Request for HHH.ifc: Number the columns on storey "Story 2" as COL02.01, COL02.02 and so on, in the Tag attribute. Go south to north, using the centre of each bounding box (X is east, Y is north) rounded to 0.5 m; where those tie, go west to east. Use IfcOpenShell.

First a look at what the model holds.

```python
import ifcopenshell
import ifcopenshell.util.element
import ifcopenshell.util.placement

model = ifcopenshell.open("HHH.ifc")
print(model.schema)
storey = next(s for s in model.by_type("IfcBuildingStorey") if s.Name == "Story 2")
columns = [e for e in ifcopenshell.util.element.get_decomposition(storey) if e.is_a("IfcColumn")]
for e in sorted(columns, key=lambda e: e.id()):
    origin = ifcopenshell.util.placement.get_local_placement(e.ObjectPlacement)[:3, 3]
    print(e.id(), e.Tag, e.Name, origin.round(2) + 0.0, sep=" | ")
```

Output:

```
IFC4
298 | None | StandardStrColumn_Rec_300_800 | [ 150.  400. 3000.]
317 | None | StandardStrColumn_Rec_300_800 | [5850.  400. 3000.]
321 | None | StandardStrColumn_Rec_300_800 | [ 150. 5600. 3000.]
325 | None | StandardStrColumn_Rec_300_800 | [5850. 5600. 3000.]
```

```python
import ifcopenshell
import ifcopenshell.geom
import ifcopenshell.util.element
import ifcopenshell.util.shape

model = ifcopenshell.open("HHH.ifc")
settings = ifcopenshell.geom.settings()
settings.set("use-world-coords", True)


def centre(element):
    shape = ifcopenshell.geom.create_shape(settings, element)
    return ifcopenshell.util.shape.get_bbox_centroid(shape.geometry)


storey = next(s for s in model.by_type("IfcBuildingStorey") if s.Name == "Story 2")
columns = [e for e in ifcopenshell.util.element.get_decomposition(storey) if e.is_a("IfcColumn")]

# Insertion points can sit at a corner or the storey origin, so sort by the geometry (in metres).
centres = {e: centre(e) for e in columns}
columns.sort(key=lambda e: (round(centres[e][1] / 0.5), centres[e][0]))

for i, e in enumerate(columns, start=1):
    number = f"COL02.{i:02d}"
    e.Tag = number
    print(e.id(), number)

model.write("HHH_v2.ifc")
```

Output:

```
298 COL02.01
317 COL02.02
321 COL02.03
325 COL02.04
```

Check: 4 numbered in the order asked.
